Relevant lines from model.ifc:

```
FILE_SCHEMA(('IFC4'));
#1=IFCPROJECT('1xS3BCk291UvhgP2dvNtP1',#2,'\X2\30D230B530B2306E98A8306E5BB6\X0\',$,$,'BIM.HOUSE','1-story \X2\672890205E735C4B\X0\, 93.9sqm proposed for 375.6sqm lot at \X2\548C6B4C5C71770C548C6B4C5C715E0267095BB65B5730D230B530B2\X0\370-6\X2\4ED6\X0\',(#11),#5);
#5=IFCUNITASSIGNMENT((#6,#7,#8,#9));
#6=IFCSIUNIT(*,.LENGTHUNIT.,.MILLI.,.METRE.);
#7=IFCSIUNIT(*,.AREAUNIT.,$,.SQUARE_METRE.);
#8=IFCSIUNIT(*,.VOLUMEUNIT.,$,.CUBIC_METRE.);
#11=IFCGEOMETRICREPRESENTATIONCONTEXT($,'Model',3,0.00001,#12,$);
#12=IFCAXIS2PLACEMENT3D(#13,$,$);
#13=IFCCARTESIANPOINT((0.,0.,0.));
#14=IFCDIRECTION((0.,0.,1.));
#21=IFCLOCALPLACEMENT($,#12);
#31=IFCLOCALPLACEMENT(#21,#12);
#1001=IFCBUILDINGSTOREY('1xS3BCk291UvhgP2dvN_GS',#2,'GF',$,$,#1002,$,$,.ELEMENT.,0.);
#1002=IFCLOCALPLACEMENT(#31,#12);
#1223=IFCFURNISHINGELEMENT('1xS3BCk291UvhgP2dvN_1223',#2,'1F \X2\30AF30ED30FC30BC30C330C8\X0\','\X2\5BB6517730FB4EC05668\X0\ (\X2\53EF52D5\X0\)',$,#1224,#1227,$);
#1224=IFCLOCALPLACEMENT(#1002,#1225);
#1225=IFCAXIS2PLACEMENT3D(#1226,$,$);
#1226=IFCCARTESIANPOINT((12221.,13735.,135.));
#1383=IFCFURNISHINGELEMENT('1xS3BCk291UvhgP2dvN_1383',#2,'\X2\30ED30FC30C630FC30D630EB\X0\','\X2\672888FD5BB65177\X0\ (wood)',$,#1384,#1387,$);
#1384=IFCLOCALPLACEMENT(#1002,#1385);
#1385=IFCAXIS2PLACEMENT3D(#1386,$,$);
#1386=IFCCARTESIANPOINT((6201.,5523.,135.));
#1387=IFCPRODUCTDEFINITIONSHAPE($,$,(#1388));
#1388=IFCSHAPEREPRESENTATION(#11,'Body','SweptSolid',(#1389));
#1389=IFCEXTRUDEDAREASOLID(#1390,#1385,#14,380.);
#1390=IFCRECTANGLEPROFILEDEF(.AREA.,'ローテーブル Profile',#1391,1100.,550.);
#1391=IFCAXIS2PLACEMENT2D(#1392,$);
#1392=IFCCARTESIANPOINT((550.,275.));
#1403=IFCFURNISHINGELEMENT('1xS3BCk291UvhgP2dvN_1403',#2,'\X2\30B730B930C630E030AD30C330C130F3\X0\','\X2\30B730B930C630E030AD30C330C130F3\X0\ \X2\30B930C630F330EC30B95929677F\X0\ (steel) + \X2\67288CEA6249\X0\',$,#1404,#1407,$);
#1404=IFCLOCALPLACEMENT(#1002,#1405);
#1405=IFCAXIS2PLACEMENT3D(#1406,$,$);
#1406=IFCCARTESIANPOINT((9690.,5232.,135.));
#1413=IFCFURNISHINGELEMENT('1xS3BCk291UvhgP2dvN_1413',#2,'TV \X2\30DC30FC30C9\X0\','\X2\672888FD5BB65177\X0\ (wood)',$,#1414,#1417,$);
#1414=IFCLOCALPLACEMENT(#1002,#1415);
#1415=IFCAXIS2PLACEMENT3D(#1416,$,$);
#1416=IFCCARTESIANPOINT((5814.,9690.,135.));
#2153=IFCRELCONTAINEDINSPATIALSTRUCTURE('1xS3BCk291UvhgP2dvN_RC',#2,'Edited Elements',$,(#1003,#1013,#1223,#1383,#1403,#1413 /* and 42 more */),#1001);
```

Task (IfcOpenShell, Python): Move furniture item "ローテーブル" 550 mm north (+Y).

```python
import ifcopenshell
import ifcopenshell.api.geometry
import ifcopenshell.util.placement

model = ifcopenshell.open("model.ifc")

item = model.by_guid("1xS3BCk291UvhgP2dvN_1383")
matrix = ifcopenshell.util.placement.get_local_placement(item.ObjectPlacement)
matrix[1, 3] += 550.0
ifcopenshell.api.geometry.edit_object_placement(model, product=item, matrix=matrix, is_si=False)

print(ifcopenshell.util.placement.get_local_placement(item.ObjectPlacement).round(3) + 0.0)

model.write("model-out.ifc")
```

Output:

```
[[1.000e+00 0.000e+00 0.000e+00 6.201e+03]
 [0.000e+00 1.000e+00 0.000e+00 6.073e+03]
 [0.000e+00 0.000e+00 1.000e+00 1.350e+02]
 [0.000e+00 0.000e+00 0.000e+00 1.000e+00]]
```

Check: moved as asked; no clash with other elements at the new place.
